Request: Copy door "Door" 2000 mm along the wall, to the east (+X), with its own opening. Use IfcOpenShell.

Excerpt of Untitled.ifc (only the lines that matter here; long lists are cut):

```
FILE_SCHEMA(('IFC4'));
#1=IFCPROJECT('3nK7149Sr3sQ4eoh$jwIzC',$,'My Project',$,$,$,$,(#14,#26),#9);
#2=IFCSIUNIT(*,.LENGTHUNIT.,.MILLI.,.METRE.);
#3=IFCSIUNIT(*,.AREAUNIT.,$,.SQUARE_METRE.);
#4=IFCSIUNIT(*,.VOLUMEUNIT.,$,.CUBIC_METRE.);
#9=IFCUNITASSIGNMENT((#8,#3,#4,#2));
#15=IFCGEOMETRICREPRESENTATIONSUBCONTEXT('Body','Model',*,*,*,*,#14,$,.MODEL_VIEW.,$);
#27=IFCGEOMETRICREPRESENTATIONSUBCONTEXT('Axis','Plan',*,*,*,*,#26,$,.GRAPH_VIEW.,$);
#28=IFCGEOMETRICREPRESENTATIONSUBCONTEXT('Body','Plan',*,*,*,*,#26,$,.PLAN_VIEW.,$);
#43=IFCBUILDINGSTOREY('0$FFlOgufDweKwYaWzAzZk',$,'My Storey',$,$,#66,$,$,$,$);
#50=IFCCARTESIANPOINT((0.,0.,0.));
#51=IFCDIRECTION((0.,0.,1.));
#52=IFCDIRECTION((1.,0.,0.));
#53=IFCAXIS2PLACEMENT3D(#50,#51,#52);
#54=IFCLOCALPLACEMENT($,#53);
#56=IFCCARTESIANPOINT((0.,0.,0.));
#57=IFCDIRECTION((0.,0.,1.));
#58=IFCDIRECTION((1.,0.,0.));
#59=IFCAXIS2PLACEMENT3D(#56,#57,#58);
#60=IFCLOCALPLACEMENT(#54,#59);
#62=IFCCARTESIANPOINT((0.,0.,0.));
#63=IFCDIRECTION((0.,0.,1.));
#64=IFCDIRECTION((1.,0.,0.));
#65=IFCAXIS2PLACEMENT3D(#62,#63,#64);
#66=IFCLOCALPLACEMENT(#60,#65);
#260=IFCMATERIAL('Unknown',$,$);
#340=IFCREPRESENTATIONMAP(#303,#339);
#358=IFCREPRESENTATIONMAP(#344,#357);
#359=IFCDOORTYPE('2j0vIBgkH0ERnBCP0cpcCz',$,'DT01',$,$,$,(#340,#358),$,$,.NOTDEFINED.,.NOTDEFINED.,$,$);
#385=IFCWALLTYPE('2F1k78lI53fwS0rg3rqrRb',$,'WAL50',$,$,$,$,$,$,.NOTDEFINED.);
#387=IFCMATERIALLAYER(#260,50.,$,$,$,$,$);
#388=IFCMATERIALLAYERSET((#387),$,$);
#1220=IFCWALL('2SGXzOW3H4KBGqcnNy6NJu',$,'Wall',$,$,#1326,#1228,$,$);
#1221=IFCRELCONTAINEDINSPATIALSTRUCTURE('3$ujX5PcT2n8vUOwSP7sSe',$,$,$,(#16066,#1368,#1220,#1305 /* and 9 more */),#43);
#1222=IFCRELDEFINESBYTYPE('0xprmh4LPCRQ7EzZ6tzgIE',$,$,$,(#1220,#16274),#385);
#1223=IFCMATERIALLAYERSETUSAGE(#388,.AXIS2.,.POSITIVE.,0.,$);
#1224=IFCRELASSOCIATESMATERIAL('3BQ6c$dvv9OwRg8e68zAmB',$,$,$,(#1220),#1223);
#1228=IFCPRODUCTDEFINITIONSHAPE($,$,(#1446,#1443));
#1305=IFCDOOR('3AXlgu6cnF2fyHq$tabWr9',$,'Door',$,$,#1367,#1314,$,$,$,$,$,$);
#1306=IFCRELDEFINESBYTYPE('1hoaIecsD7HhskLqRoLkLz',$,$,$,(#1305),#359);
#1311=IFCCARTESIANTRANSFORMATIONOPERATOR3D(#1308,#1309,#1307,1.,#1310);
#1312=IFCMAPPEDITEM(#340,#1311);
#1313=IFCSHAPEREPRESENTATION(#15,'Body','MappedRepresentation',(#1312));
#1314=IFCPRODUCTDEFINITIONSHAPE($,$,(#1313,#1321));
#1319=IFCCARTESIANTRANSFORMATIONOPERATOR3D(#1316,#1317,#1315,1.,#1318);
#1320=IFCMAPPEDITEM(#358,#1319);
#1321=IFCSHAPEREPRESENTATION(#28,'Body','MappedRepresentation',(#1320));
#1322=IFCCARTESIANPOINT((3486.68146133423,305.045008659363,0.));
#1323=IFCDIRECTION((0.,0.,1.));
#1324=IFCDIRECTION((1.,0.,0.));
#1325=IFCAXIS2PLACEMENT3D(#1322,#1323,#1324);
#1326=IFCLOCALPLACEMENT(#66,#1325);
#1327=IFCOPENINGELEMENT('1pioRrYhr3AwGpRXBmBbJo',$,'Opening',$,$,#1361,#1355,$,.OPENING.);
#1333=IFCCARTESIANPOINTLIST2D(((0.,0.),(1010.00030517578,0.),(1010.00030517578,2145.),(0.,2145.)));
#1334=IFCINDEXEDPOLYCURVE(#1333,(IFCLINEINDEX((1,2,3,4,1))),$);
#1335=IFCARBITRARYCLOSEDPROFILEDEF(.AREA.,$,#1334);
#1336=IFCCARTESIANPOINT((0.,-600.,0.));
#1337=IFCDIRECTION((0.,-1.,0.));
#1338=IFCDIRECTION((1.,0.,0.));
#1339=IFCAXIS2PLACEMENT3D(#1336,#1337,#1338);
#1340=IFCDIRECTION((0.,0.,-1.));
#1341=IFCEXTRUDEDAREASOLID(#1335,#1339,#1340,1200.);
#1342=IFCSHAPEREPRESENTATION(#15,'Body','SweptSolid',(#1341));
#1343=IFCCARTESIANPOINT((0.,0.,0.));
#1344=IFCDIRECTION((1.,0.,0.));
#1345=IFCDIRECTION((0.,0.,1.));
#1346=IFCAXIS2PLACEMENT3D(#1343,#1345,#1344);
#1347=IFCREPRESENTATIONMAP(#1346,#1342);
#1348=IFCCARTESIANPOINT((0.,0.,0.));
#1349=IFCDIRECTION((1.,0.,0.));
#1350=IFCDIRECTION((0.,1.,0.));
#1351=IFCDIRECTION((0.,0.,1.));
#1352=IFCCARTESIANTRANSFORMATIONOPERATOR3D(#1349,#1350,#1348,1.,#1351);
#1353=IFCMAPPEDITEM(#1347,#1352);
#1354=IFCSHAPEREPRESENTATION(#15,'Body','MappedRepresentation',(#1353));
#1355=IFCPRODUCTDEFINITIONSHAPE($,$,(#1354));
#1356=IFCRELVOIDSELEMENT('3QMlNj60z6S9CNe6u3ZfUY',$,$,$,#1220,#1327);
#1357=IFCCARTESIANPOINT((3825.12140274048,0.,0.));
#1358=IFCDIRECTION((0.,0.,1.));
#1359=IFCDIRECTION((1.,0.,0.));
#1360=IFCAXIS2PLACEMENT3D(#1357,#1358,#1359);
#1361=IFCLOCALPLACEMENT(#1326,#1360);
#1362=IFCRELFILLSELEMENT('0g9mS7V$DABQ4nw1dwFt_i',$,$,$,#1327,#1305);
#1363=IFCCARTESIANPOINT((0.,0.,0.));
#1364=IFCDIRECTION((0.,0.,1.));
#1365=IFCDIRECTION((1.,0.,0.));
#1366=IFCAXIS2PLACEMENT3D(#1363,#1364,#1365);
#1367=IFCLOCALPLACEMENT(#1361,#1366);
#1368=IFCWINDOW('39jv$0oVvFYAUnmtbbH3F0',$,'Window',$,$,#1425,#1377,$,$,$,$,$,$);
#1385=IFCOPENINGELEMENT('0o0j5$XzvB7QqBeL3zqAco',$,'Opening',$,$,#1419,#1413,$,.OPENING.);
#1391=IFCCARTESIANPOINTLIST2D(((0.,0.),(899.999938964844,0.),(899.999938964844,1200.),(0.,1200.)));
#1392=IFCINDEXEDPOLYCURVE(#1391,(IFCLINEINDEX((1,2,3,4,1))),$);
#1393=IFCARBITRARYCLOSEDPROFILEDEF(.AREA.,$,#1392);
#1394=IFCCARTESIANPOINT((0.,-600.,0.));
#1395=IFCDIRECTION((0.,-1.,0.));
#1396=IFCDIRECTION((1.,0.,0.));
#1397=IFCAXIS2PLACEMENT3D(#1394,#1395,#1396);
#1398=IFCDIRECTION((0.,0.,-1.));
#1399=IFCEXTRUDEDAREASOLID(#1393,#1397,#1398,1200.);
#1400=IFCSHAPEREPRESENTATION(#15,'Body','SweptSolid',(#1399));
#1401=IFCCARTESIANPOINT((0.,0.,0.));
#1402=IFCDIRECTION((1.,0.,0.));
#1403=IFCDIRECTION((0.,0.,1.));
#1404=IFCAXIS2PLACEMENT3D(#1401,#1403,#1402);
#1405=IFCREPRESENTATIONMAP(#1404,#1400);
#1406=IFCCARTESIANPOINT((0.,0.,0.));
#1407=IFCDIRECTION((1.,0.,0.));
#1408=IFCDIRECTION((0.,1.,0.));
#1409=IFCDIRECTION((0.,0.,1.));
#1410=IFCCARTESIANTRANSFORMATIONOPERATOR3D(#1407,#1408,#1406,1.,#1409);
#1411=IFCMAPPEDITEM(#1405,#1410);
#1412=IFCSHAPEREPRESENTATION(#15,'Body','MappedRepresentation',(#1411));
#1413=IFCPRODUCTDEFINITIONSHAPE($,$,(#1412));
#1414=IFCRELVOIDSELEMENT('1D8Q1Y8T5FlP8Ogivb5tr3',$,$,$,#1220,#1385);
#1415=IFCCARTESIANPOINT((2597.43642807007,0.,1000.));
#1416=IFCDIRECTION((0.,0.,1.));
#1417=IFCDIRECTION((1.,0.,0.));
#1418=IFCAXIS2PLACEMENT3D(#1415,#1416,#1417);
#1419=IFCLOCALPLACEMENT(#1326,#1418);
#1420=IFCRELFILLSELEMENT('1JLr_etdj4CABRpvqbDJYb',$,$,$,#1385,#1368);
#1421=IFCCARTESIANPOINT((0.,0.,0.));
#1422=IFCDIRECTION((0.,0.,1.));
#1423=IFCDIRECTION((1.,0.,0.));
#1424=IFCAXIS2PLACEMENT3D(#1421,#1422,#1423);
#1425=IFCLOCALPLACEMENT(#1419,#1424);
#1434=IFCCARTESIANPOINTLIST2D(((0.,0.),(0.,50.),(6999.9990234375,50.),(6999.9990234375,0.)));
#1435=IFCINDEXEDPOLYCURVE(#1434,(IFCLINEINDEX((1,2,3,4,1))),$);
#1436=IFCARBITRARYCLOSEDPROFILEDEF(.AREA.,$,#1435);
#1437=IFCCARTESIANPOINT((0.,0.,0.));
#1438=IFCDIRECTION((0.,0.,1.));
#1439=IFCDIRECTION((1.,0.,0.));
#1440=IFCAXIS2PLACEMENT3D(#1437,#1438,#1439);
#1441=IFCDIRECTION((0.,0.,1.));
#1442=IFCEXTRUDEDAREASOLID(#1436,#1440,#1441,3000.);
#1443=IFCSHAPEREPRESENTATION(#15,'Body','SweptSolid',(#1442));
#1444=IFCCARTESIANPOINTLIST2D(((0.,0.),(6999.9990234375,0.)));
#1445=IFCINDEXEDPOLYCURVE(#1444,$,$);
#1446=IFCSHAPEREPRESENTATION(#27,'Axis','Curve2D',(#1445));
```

```python
import ifcopenshell
import ifcopenshell.api.feature
import ifcopenshell.api.geometry
import ifcopenshell.api.root
import ifcopenshell.geom
import ifcopenshell.util.element
import ifcopenshell.util.placement
import ifcopenshell.util.shape

model = ifcopenshell.open("Untitled.ifc")
settings = ifcopenshell.geom.settings()


def volume(element):
    """Net volume in cubic metres, openings subtracted."""
    shape = ifcopenshell.geom.create_shape(settings, element)
    return ifcopenshell.util.shape.get_volume(shape.geometry)


door = model.by_guid("3AXlgu6cnF2fyHq$tabWr9")
opening = door.FillsVoids[0].RelatingOpeningElement
wall = opening.VoidsElements[0].RelatingBuildingElement
before = volume(wall)
shift = ifcopenshell.util.placement.get_local_placement(wall.ObjectPlacement)[:3, 0] * 2000.0

# copy_class copies the void relationship, type, container and properties, but no geometry.
new_opening = ifcopenshell.api.root.copy_class(model, product=opening)
new_opening.Representation = ifcopenshell.util.element.copy_deep(
    model, opening.Representation, exclude=["IfcGeometricRepresentationContext", "IfcRepresentationMap"]
)
new_door = ifcopenshell.api.root.copy_class(model, product=door)
new_door.Representation = ifcopenshell.util.element.copy_deep(
    model, door.Representation, exclude=["IfcGeometricRepresentationContext", "IfcRepresentationMap"]
)
ifcopenshell.api.feature.add_filling(model, opening=new_opening, element=new_door)

for old, new in ((opening, new_opening), (door, new_door)):
    matrix = ifcopenshell.util.placement.get_local_placement(old.ObjectPlacement)
    matrix[:3, 3] += shift
    ifcopenshell.api.geometry.edit_object_placement(model, product=new, matrix=matrix, is_si=False)

after = volume(wall)

print(f"wall volume {before:.3f} -> {after:.3f} m3")

model.write("Untitled-out.ifc")
```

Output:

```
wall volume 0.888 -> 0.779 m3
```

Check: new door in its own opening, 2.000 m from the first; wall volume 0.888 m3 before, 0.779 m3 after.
